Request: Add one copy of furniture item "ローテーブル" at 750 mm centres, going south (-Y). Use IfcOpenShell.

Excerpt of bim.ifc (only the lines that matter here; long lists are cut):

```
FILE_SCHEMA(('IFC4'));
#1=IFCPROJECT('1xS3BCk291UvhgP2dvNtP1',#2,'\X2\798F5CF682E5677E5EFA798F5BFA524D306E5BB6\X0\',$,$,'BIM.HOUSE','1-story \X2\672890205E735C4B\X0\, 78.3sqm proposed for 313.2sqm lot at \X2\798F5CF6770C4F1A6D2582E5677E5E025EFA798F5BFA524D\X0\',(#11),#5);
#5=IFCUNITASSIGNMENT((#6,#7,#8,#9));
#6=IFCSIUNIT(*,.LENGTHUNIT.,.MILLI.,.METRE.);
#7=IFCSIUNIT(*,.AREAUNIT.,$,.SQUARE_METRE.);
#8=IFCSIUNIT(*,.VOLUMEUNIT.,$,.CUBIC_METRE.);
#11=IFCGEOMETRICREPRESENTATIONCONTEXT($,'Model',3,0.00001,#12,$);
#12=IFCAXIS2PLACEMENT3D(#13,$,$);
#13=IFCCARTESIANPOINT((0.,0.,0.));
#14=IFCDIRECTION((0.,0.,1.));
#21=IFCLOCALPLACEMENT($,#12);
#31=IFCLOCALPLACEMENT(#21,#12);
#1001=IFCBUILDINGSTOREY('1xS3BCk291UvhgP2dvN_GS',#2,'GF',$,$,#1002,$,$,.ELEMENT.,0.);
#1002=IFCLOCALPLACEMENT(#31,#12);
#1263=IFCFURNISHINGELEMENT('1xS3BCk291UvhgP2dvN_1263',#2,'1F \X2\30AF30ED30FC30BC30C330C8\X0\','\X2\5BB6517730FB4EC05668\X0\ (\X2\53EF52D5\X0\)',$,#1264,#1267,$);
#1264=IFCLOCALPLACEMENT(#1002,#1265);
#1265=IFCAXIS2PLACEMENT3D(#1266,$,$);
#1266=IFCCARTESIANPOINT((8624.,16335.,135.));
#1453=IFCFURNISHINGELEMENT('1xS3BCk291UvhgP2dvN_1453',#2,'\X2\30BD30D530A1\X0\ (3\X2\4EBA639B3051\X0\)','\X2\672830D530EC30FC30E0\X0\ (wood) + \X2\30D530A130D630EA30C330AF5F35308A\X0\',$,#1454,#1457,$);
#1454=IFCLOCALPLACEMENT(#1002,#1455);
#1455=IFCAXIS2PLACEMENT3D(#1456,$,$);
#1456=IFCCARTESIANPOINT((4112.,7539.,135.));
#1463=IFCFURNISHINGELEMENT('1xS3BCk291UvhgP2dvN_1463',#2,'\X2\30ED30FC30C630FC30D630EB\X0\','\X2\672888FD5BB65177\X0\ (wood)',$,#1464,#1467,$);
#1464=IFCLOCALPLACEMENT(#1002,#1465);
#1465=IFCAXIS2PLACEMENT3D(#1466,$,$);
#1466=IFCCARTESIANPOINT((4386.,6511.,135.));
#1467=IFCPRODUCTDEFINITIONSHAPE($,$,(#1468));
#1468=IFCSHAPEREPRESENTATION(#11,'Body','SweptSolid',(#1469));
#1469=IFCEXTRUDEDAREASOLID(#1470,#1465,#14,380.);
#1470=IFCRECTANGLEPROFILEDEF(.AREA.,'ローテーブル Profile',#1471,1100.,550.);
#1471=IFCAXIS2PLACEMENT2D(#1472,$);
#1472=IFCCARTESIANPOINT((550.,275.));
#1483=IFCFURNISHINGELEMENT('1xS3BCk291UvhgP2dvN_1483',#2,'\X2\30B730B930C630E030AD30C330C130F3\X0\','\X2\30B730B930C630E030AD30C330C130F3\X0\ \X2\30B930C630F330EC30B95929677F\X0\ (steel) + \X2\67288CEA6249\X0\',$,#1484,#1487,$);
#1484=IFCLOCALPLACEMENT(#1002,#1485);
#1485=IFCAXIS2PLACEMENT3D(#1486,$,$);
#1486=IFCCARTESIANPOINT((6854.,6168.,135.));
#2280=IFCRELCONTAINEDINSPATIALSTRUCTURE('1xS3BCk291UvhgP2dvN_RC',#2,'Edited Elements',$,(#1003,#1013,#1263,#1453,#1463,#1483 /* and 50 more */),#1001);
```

```python
import numpy as np
import ifcopenshell
import ifcopenshell.api.geometry
import ifcopenshell.api.root
import ifcopenshell.util.element
import ifcopenshell.util.placement

model = ifcopenshell.open("bim.ifc")


def reuse_history(source, copy):
    """copy_class also copies each property set's owner history, people and application; keep the originals."""
    for rel in copy.IsDefinedBy:
        if rel.is_a("IfcRelDefinesByProperties") and (history := rel.RelatingPropertyDefinition.OwnerHistory):
            rel.RelatingPropertyDefinition.OwnerHistory = source.OwnerHistory
            ifcopenshell.util.element.remove_deep2(model, history)


source = model.by_guid("1xS3BCk291UvhgP2dvN_1463")
base = ifcopenshell.util.placement.get_local_placement(source.ObjectPlacement)
step = np.array([0.0, -1.0, 0.0]) * 750.0

for i in range(1, 2):
    copy = ifcopenshell.api.root.copy_class(model, product=source)
    copy.Representation = ifcopenshell.util.element.copy_deep(
        model, source.Representation, exclude=["IfcGeometricRepresentationContext", "IfcRepresentationMap"]
    )
    reuse_history(source, copy)
    matrix = base.copy()
    matrix[:3, 3] += i * step
    print("added at", matrix[:3, 3].round(3) + 0.0)
    ifcopenshell.api.geometry.edit_object_placement(model, product=copy, matrix=matrix, is_si=False)

model.write("bim_updated.ifc")
```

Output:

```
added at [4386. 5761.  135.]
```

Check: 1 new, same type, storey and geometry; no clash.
